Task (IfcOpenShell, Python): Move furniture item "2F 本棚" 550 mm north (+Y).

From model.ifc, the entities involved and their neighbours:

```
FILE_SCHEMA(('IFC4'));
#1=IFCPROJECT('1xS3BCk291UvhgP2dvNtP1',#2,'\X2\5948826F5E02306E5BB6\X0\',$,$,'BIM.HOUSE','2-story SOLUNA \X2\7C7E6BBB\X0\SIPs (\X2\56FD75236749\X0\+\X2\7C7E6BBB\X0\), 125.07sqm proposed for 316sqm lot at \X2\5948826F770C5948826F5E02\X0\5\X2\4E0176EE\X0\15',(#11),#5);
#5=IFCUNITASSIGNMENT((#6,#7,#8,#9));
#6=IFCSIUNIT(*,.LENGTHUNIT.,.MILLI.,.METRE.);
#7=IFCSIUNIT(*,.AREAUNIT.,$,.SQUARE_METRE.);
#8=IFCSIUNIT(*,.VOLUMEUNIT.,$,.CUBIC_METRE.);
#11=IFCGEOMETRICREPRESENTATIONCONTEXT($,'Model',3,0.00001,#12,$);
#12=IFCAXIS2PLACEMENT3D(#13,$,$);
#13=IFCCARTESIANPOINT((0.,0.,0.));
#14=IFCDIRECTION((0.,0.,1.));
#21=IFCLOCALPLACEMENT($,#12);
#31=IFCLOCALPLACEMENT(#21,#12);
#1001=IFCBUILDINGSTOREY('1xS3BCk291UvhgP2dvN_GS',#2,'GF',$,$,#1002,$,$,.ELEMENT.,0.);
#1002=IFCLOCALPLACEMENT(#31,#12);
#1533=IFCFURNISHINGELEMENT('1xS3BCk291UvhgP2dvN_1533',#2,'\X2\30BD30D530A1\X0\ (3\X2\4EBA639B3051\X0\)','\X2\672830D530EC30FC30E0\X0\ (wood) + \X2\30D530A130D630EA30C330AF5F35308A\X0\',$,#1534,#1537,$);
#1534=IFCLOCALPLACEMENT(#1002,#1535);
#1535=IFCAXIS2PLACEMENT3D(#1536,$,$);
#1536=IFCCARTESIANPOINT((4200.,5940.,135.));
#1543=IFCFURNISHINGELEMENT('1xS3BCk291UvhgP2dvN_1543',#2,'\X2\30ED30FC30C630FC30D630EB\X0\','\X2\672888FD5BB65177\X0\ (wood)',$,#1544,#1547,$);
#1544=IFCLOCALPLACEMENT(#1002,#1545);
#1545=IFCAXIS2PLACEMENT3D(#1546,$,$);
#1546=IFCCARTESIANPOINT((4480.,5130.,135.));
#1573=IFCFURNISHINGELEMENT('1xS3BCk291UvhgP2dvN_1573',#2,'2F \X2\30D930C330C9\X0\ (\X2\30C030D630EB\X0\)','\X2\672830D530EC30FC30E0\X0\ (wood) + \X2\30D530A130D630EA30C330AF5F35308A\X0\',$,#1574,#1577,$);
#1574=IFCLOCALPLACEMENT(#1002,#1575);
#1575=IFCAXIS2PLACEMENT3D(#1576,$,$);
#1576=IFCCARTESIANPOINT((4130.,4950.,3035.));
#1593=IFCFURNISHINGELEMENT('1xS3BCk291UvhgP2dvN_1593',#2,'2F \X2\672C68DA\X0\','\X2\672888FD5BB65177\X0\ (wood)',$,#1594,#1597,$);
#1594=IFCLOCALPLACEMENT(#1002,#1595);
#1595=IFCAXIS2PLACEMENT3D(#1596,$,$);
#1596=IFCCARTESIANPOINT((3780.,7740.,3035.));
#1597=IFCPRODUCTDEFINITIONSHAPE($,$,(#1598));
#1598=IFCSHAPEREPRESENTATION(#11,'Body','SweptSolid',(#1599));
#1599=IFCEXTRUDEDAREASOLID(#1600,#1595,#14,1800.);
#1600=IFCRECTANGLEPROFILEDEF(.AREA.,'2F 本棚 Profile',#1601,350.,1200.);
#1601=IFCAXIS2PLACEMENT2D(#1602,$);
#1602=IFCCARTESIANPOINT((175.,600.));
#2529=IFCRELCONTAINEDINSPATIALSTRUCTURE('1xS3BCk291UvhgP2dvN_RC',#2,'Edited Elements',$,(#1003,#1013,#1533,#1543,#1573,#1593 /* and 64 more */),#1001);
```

```python
import ifcopenshell
import ifcopenshell.api.geometry
import ifcopenshell.util.placement
import ifcopenshell.util.unit

model = ifcopenshell.open("model.ifc")
unit_scale = ifcopenshell.util.unit.calculate_unit_scale(model)

item = model.by_guid("1xS3BCk291UvhgP2dvN_1593")
matrix = ifcopenshell.util.placement.get_local_placement(item.ObjectPlacement)
matrix[1, 3] += 0.55 / unit_scale
ifcopenshell.api.geometry.edit_object_placement(model, product=item, matrix=matrix, is_si=False)

print(ifcopenshell.util.placement.get_local_placement(item.ObjectPlacement).round(3) + 0.0)

model.write("model_v2.ifc")
```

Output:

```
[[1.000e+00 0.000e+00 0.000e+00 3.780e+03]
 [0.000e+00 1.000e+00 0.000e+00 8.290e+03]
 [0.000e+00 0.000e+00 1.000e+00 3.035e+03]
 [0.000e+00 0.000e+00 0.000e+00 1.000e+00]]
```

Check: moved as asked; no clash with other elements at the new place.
